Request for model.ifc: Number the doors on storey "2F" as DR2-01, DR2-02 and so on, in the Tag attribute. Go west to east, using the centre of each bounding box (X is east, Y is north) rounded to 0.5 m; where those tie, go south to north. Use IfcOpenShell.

First a look at what the model holds.

```python
import ifcopenshell
import ifcopenshell.util.element
import ifcopenshell.util.placement

model = ifcopenshell.open("model.ifc")
print(model.schema)
storey = next(s for s in model.by_type("IfcBuildingStorey") if s.Name == "2F")
doors = [e for e in ifcopenshell.util.element.get_decomposition(storey) if e.is_a("IfcDoor")]
for e in sorted(doors, key=lambda e: e.id()):
    origin = ifcopenshell.util.placement.get_local_placement(e.ObjectPlacement)[:3, 3]
    print(e.id(), e.Tag, e.Name, origin.round(2) + 0.0, sep=" | ")
```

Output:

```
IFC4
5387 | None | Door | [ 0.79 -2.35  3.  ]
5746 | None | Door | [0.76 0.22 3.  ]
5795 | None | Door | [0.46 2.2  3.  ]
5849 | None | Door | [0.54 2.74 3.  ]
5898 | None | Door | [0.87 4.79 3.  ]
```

```python
import ifcopenshell
import ifcopenshell.geom
import ifcopenshell.util.element
import ifcopenshell.util.shape

model = ifcopenshell.open("model.ifc")
settings = ifcopenshell.geom.settings()
settings.set("use-world-coords", True)


def centre(element):
    shape = ifcopenshell.geom.create_shape(settings, element)
    return ifcopenshell.util.shape.get_bbox_centroid(shape.geometry)


storey = next(s for s in model.by_type("IfcBuildingStorey") if s.Name == "2F")
doors = [e for e in ifcopenshell.util.element.get_decomposition(storey) if e.is_a("IfcDoor")]

# Insertion points can sit at a corner or the storey origin, so sort by the geometry (in metres).
centres = {e: centre(e) for e in doors}
doors.sort(key=lambda e: (round(centres[e][0] / 0.5), centres[e][1]))

for i, e in enumerate(doors, start=1):
    number = f"DR2-{i:02d}"
    e.Tag = number
    print(e.id(), number)

model.write("model_rev.ifc")
```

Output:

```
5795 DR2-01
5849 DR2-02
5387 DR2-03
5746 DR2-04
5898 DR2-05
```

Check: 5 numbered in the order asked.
